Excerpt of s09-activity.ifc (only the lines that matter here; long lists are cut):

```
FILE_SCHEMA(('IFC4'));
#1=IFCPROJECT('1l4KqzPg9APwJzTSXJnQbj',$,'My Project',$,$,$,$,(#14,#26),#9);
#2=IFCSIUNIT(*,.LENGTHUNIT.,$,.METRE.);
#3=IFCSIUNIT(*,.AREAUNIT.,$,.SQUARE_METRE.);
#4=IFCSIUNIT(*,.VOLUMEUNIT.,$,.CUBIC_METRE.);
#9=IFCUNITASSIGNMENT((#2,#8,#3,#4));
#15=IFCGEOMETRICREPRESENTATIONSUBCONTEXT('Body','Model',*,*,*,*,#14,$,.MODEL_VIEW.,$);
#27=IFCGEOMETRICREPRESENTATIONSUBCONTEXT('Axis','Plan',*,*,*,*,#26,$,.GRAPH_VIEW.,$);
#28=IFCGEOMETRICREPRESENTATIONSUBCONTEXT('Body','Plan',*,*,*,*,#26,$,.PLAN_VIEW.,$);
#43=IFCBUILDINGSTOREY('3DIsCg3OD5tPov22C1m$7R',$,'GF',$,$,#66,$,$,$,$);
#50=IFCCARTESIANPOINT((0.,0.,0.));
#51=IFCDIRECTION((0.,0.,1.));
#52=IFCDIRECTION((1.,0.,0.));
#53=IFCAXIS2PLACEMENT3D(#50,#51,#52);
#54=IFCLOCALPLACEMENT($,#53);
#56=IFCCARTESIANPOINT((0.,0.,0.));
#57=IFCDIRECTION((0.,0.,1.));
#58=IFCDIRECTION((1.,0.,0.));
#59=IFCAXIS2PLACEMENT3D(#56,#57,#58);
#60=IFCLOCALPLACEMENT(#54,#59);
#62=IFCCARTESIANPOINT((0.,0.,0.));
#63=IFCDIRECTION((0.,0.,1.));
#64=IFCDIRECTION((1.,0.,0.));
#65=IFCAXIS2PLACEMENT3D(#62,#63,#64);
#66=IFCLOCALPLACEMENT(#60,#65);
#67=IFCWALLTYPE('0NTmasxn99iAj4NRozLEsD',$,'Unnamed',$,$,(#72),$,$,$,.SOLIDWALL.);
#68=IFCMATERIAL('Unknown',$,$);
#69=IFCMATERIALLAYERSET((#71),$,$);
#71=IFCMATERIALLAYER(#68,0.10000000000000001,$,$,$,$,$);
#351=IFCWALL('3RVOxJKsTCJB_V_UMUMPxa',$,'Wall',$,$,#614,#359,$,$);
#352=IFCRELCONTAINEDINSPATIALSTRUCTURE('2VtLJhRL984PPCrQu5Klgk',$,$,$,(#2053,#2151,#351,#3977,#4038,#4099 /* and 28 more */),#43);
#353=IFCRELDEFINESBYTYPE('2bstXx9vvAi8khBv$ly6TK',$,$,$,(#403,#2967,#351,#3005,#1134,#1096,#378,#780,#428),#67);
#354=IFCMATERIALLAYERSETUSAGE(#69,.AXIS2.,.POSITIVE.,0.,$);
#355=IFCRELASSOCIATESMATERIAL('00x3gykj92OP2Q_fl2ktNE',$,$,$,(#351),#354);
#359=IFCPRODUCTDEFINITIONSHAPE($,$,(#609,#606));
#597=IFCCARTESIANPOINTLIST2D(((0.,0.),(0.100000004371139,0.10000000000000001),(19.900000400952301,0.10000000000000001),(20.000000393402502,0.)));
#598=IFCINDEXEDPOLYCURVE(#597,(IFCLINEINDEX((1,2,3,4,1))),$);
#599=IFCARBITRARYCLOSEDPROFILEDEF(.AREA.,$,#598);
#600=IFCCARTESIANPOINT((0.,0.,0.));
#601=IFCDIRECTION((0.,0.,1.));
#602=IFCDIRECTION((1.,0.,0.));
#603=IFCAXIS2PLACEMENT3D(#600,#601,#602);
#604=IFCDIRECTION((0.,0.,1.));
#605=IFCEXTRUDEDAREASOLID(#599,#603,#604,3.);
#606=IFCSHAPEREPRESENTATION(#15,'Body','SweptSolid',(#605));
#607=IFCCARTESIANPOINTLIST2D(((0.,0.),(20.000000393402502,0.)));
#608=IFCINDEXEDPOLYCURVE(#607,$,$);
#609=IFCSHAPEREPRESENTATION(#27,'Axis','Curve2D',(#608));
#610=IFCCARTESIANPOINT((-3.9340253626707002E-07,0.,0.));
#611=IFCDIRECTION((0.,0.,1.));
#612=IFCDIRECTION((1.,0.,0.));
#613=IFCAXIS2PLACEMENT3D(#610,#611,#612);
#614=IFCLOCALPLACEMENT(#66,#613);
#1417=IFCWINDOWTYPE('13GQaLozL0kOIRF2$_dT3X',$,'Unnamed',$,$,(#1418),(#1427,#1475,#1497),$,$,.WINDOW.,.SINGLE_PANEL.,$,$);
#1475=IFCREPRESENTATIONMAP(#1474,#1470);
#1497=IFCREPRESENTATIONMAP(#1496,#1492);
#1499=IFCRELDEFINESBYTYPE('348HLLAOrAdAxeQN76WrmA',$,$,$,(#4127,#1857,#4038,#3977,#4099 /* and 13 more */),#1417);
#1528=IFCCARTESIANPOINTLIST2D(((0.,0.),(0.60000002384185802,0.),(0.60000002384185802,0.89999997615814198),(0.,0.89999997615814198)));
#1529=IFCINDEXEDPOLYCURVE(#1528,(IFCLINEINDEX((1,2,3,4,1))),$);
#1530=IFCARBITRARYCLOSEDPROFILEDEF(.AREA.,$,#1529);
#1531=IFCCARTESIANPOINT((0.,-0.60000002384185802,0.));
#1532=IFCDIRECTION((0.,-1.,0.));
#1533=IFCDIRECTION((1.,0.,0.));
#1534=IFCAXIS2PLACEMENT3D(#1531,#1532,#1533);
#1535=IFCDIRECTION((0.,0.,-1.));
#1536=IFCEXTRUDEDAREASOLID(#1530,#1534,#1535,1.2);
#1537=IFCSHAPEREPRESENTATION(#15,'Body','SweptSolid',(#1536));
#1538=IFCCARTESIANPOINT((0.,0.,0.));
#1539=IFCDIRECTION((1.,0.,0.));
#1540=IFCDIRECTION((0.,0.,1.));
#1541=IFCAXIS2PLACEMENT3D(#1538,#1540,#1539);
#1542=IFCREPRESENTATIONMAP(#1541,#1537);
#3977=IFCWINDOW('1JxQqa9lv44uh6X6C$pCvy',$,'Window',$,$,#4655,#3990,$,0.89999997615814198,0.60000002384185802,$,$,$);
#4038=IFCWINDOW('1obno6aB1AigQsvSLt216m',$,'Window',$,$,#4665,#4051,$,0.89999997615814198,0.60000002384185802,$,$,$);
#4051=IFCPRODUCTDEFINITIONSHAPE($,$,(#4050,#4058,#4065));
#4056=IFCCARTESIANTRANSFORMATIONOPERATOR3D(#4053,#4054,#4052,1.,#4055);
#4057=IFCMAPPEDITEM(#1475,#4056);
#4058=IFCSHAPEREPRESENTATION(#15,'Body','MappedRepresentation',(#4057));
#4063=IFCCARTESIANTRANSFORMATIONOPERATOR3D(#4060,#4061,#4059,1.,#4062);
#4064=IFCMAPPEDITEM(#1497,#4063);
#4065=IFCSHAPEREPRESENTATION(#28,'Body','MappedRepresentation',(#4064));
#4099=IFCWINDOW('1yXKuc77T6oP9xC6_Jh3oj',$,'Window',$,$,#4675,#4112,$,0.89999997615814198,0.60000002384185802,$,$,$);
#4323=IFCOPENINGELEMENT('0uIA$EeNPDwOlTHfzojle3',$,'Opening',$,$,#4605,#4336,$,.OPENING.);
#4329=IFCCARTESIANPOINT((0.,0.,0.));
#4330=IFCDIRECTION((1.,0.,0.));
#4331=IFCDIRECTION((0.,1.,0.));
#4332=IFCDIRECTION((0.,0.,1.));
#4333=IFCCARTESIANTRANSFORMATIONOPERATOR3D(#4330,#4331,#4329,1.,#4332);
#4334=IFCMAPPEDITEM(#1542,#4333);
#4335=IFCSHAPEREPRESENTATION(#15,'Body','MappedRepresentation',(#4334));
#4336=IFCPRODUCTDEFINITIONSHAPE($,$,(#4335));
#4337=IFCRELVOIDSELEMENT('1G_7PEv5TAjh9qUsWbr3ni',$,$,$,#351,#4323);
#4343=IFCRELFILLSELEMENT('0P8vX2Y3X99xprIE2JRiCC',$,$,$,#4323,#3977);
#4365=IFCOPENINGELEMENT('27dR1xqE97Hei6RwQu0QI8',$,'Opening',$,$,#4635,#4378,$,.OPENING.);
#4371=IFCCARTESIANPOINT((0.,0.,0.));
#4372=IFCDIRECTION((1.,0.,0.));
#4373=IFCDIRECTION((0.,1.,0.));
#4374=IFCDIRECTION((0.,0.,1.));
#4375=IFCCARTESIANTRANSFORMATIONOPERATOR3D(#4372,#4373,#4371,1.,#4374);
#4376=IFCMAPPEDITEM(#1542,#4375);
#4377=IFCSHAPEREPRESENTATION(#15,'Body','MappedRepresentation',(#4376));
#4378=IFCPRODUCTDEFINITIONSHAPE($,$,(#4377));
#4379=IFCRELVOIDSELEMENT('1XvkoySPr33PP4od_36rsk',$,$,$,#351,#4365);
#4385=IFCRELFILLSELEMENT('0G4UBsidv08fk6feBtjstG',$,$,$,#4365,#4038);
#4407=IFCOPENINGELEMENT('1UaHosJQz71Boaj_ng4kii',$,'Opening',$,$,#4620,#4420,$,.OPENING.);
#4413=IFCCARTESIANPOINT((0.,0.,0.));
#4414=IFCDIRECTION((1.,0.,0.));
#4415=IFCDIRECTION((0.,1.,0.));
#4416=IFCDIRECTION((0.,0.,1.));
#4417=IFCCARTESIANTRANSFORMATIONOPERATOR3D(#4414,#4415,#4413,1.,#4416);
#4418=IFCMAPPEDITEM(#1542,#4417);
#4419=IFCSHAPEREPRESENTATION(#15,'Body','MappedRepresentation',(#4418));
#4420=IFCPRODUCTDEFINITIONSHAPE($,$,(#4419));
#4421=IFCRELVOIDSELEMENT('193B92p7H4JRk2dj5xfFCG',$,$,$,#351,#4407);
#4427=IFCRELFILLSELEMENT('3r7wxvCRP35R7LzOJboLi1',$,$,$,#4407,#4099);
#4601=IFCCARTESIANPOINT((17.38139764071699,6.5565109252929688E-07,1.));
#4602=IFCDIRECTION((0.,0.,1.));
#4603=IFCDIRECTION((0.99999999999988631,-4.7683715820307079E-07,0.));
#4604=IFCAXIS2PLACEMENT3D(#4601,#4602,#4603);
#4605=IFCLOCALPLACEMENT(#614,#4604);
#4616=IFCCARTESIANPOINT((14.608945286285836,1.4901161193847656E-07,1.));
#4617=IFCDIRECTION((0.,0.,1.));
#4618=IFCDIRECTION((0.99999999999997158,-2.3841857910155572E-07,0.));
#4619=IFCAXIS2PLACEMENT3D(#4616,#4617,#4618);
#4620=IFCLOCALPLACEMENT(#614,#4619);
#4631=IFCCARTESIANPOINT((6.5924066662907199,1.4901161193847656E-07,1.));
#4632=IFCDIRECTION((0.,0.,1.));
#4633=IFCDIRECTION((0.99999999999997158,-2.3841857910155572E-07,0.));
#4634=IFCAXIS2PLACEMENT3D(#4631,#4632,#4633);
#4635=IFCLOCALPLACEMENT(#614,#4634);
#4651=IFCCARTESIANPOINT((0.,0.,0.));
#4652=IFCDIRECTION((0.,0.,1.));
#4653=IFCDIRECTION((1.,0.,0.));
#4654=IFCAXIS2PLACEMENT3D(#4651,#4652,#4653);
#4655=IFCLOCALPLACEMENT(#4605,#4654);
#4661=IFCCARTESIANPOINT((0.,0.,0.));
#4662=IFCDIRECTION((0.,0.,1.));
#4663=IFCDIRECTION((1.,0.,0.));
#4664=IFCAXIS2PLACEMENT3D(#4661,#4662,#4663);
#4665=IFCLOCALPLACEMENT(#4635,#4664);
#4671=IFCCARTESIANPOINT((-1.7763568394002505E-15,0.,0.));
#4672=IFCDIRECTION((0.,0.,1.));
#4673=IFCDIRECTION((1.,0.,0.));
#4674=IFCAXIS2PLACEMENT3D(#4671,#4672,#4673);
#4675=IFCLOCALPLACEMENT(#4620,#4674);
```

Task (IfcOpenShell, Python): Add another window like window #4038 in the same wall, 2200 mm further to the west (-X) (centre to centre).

```python
import ifcopenshell
import ifcopenshell.api.feature
import ifcopenshell.api.geometry
import ifcopenshell.api.root
import ifcopenshell.geom
import ifcopenshell.util.element
import ifcopenshell.util.placement
import ifcopenshell.util.shape

model = ifcopenshell.open("s09-activity.ifc")
settings = ifcopenshell.geom.settings()


def volume(element):
    """Net volume in cubic metres, openings subtracted."""
    shape = ifcopenshell.geom.create_shape(settings, element)
    return ifcopenshell.util.shape.get_volume(shape.geometry)


window = model.by_guid("1obno6aB1AigQsvSLt216m")
opening = window.FillsVoids[0].RelatingOpeningElement
wall = opening.VoidsElements[0].RelatingBuildingElement
before = volume(wall)
shift = ifcopenshell.util.placement.get_local_placement(wall.ObjectPlacement)[:3, 0] * -2.2

# copy_class copies the void relationship, type, container and properties, but no geometry.
new_opening = ifcopenshell.api.root.copy_class(model, product=opening)
new_opening.Representation = ifcopenshell.util.element.copy_deep(
    model, opening.Representation, exclude=["IfcGeometricRepresentationContext", "IfcRepresentationMap"]
)
new_window = ifcopenshell.api.root.copy_class(model, product=window)
new_window.Representation = ifcopenshell.util.element.copy_deep(
    model, window.Representation, exclude=["IfcGeometricRepresentationContext", "IfcRepresentationMap"]
)
ifcopenshell.api.feature.add_filling(model, opening=new_opening, element=new_window)

for old, new in ((opening, new_opening), (window, new_window)):
    matrix = ifcopenshell.util.placement.get_local_placement(old.ObjectPlacement)
    matrix[:3, 3] += shift
    ifcopenshell.api.geometry.edit_object_placement(model, product=new, matrix=matrix, is_si=False)

after = volume(wall)

print(f"wall volume {before:.3f} -> {after:.3f} m3")

model.write("s09-activity-out.ifc")
```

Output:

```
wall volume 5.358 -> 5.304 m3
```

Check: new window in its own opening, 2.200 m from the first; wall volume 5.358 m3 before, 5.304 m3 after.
